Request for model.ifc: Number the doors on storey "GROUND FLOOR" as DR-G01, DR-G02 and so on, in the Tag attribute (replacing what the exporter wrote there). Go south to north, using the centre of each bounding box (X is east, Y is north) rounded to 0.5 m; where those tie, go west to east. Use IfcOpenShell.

First a look at what the model holds.

```python
import ifcopenshell
import ifcopenshell.util.element
import ifcopenshell.util.placement

model = ifcopenshell.open("model.ifc")
print(model.schema)
storey = next(s for s in model.by_type("IfcBuildingStorey") if s.Name == "GROUND FLOOR")
doors = [e for e in ifcopenshell.util.element.get_decomposition(storey) if e.is_a("IfcDoor")]
for e in sorted(doors, key=lambda e: e.id()):
    origin = ifcopenshell.util.placement.get_local_placement(e.ObjectPlacement)[:3, 3]
    print(e.id(), e.Tag, e.Name, origin.round(2) + 0.0, sep=" | ")
```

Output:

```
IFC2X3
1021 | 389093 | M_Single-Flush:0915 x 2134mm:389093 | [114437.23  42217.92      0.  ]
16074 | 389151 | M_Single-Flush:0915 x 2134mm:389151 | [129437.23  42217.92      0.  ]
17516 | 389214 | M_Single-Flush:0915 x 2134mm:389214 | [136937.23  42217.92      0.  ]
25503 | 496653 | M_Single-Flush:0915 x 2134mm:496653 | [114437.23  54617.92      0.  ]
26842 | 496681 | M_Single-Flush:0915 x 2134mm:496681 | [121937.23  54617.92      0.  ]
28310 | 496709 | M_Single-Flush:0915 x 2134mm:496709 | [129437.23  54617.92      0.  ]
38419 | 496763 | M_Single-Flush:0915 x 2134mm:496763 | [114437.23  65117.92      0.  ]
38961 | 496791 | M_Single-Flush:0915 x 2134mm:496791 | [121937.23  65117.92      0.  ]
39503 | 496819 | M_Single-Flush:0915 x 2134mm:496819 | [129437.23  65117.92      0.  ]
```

```python
import ifcopenshell
import ifcopenshell.geom
import ifcopenshell.util.element
import ifcopenshell.util.shape

model = ifcopenshell.open("model.ifc")
settings = ifcopenshell.geom.settings()
settings.set("use-world-coords", True)


def centre(element):
    shape = ifcopenshell.geom.create_shape(settings, element)
    return ifcopenshell.util.shape.get_bbox_centroid(shape.geometry)


storey = next(s for s in model.by_type("IfcBuildingStorey") if s.Name == "GROUND FLOOR")
doors = [e for e in ifcopenshell.util.element.get_decomposition(storey) if e.is_a("IfcDoor")]

# Insertion points can sit at a corner or the storey origin, so sort by the geometry (in metres).
centres = {e: centre(e) for e in doors}
doors.sort(key=lambda e: (round(centres[e][1] / 0.5), centres[e][0]))

for i, e in enumerate(doors, start=1):
    number = f"DR-G{i:02d}"
    e.Tag = number
    print(e.id(), number)

model.write("model_v2.ifc")
```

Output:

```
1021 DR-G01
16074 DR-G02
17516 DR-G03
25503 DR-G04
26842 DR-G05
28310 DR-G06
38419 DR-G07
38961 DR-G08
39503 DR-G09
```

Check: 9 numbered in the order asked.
